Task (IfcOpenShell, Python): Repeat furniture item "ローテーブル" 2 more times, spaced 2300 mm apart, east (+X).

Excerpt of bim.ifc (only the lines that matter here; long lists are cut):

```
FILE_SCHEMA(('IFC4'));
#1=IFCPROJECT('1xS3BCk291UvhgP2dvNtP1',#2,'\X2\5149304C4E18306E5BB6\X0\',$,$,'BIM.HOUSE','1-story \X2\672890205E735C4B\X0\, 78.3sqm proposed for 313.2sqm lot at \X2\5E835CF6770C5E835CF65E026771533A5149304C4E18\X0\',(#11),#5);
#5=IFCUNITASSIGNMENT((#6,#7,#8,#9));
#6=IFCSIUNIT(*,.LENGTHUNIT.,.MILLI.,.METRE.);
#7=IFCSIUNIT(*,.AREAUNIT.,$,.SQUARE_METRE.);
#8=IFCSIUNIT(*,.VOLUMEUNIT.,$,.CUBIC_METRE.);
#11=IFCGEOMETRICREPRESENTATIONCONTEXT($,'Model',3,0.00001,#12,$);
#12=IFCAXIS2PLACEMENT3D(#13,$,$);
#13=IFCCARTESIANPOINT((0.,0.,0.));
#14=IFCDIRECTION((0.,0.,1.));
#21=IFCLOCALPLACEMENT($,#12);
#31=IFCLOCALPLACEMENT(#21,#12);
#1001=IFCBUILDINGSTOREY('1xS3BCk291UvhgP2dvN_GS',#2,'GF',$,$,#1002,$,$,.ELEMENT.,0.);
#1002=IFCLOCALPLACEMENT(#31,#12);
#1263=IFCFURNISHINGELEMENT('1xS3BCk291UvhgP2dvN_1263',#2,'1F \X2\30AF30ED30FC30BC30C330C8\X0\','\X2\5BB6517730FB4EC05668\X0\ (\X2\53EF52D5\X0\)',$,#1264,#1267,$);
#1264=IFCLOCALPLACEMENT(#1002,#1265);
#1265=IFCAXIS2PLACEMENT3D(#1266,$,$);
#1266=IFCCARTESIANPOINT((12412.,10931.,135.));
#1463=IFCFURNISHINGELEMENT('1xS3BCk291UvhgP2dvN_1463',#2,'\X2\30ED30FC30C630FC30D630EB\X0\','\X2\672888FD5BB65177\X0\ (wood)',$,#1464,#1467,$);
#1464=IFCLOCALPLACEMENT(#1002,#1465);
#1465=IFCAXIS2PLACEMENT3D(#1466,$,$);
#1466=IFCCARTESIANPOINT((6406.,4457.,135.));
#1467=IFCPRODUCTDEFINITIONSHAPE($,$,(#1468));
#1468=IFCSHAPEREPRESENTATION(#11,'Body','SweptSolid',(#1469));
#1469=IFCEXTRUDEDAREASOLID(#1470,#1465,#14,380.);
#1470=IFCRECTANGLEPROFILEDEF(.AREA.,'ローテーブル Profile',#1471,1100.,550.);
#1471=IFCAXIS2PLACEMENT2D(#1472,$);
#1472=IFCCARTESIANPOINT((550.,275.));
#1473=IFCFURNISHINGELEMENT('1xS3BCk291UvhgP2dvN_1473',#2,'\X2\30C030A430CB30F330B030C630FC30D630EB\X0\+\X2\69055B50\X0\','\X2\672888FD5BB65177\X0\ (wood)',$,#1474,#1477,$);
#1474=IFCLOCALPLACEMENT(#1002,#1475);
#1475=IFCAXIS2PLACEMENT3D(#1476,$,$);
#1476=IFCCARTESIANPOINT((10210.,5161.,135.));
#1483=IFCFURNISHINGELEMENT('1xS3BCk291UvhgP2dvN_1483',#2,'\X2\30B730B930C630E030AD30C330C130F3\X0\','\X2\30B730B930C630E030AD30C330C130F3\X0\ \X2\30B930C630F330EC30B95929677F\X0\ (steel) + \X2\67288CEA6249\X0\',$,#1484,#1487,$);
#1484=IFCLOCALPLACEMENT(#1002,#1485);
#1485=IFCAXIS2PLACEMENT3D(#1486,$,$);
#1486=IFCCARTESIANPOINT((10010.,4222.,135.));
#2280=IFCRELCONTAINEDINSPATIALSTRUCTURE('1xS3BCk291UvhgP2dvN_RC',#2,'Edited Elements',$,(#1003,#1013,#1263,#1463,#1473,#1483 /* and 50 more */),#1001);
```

```python
import numpy as np
import ifcopenshell
import ifcopenshell.api.geometry
import ifcopenshell.api.root
import ifcopenshell.util.element
import ifcopenshell.util.placement
import ifcopenshell.util.unit

model = ifcopenshell.open("bim.ifc")
unit_scale = ifcopenshell.util.unit.calculate_unit_scale(model)


def reuse_history(source, copy):
    """copy_class also copies each property set's owner history, people and application; keep the originals."""
    for rel in copy.IsDefinedBy:
        if rel.is_a("IfcRelDefinesByProperties") and (history := rel.RelatingPropertyDefinition.OwnerHistory):
            rel.RelatingPropertyDefinition.OwnerHistory = source.OwnerHistory
            ifcopenshell.util.element.remove_deep2(model, history)


source = model.by_id(1463)
base = ifcopenshell.util.placement.get_local_placement(source.ObjectPlacement)
step = np.array([1.0, 0.0, 0.0]) * 2.3 / unit_scale

for i in range(1, 3):
    copy = ifcopenshell.api.root.copy_class(model, product=source)
    copy.Representation = ifcopenshell.util.element.copy_deep(
        model, source.Representation, exclude=["IfcGeometricRepresentationContext", "IfcRepresentationMap"]
    )
    reuse_history(source, copy)
    matrix = base.copy()
    matrix[:3, 3] += i * step
    print("added at", matrix[:3, 3].round(3) + 0.0)
    ifcopenshell.api.geometry.edit_object_placement(model, product=copy, matrix=matrix, is_si=False)

model.write("bim_rev.ifc")
```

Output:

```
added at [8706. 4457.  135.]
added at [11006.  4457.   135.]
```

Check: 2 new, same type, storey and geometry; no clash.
